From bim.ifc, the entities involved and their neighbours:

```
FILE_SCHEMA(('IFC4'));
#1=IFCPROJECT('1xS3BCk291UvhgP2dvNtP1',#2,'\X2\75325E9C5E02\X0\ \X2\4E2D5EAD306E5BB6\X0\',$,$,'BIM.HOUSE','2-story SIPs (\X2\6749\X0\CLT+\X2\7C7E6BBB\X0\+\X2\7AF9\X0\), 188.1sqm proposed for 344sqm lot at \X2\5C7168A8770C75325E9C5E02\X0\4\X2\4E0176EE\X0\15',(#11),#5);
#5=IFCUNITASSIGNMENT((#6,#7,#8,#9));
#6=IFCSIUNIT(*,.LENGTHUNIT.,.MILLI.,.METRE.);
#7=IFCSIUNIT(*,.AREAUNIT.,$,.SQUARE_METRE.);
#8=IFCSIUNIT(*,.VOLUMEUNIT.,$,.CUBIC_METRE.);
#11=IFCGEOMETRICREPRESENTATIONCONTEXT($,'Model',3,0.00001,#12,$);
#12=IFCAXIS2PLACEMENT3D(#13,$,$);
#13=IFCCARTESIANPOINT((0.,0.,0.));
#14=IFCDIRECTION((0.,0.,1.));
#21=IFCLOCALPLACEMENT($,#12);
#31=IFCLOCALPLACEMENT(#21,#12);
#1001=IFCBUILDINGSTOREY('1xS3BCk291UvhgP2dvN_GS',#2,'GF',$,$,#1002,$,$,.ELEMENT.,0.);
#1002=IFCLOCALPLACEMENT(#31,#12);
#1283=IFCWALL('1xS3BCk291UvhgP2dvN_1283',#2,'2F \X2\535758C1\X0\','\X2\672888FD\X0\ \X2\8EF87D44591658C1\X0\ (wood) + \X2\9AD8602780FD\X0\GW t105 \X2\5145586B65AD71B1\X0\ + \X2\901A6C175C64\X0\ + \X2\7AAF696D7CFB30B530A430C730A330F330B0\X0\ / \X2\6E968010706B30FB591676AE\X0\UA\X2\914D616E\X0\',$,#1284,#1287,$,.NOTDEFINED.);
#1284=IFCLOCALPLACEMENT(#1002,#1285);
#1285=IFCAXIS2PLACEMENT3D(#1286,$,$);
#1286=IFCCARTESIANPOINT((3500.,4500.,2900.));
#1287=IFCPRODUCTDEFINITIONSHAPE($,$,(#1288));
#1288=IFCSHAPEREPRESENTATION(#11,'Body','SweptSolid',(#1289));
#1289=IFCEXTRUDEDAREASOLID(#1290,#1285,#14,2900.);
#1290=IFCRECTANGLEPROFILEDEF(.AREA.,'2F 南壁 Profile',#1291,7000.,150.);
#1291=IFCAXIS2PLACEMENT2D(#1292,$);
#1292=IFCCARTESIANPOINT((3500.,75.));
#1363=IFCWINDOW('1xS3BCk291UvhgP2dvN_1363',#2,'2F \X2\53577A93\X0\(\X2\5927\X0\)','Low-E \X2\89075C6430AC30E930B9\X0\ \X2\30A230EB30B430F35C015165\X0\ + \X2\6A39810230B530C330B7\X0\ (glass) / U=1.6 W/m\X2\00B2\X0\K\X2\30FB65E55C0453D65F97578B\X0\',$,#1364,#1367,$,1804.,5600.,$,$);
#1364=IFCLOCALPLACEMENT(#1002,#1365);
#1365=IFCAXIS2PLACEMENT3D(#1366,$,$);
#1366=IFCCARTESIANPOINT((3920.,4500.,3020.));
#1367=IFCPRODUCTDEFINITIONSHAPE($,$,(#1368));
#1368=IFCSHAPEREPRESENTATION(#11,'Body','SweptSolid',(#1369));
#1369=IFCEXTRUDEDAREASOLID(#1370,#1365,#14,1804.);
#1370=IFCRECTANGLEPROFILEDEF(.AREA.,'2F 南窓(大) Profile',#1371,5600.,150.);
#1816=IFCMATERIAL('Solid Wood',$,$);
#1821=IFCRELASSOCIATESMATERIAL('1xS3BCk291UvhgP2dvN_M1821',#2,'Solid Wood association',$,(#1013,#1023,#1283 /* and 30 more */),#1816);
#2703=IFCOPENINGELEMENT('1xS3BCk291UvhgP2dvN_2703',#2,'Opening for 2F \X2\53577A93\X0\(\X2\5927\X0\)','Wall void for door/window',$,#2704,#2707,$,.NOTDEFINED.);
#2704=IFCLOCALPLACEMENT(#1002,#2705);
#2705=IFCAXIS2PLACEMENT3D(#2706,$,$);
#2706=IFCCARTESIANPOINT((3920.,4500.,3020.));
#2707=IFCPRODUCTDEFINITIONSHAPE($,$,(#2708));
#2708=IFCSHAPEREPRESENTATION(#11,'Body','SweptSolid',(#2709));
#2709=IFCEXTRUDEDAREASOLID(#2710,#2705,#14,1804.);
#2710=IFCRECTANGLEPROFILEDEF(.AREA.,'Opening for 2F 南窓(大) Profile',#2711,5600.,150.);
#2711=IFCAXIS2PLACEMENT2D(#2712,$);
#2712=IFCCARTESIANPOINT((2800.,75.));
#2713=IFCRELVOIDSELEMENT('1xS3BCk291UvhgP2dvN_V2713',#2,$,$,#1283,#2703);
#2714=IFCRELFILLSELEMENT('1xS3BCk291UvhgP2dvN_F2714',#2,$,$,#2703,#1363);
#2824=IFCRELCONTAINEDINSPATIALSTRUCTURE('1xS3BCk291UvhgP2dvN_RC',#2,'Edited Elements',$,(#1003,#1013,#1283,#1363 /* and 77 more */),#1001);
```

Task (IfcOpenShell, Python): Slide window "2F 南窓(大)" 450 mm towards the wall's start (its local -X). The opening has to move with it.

```python
import ifcopenshell
import ifcopenshell.api.geometry
import ifcopenshell.util.placement
import ifcopenshell.util.unit

model = ifcopenshell.open("bim.ifc")
unit_scale = ifcopenshell.util.unit.calculate_unit_scale(model)

window = model.by_guid("1xS3BCk291UvhgP2dvN_1363")
opening = window.FillsVoids[0].RelatingOpeningElement
wall = opening.VoidsElements[0].RelatingBuildingElement

wall_matrix = ifcopenshell.util.placement.get_local_placement(wall.ObjectPlacement)
shift = wall_matrix[:3, 0] * -0.45 / unit_scale
before = ifcopenshell.util.placement.get_local_placement(window.ObjectPlacement)[:3, 3].copy()

# The window is not placed relative to its opening, so move both.
for product in (opening, window):
    matrix = ifcopenshell.util.placement.get_local_placement(product.ObjectPlacement)
    matrix[:3, 3] += shift
    ifcopenshell.api.geometry.edit_object_placement(model, product=product, matrix=matrix, is_si=False)

after = ifcopenshell.util.placement.get_local_placement(window.ObjectPlacement)[:3, 3]
print("window moved by", (after - before).round(3) + 0.0)

model.write("bim-out.ifc")
```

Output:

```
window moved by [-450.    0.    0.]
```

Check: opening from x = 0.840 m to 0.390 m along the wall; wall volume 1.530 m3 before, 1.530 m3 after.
